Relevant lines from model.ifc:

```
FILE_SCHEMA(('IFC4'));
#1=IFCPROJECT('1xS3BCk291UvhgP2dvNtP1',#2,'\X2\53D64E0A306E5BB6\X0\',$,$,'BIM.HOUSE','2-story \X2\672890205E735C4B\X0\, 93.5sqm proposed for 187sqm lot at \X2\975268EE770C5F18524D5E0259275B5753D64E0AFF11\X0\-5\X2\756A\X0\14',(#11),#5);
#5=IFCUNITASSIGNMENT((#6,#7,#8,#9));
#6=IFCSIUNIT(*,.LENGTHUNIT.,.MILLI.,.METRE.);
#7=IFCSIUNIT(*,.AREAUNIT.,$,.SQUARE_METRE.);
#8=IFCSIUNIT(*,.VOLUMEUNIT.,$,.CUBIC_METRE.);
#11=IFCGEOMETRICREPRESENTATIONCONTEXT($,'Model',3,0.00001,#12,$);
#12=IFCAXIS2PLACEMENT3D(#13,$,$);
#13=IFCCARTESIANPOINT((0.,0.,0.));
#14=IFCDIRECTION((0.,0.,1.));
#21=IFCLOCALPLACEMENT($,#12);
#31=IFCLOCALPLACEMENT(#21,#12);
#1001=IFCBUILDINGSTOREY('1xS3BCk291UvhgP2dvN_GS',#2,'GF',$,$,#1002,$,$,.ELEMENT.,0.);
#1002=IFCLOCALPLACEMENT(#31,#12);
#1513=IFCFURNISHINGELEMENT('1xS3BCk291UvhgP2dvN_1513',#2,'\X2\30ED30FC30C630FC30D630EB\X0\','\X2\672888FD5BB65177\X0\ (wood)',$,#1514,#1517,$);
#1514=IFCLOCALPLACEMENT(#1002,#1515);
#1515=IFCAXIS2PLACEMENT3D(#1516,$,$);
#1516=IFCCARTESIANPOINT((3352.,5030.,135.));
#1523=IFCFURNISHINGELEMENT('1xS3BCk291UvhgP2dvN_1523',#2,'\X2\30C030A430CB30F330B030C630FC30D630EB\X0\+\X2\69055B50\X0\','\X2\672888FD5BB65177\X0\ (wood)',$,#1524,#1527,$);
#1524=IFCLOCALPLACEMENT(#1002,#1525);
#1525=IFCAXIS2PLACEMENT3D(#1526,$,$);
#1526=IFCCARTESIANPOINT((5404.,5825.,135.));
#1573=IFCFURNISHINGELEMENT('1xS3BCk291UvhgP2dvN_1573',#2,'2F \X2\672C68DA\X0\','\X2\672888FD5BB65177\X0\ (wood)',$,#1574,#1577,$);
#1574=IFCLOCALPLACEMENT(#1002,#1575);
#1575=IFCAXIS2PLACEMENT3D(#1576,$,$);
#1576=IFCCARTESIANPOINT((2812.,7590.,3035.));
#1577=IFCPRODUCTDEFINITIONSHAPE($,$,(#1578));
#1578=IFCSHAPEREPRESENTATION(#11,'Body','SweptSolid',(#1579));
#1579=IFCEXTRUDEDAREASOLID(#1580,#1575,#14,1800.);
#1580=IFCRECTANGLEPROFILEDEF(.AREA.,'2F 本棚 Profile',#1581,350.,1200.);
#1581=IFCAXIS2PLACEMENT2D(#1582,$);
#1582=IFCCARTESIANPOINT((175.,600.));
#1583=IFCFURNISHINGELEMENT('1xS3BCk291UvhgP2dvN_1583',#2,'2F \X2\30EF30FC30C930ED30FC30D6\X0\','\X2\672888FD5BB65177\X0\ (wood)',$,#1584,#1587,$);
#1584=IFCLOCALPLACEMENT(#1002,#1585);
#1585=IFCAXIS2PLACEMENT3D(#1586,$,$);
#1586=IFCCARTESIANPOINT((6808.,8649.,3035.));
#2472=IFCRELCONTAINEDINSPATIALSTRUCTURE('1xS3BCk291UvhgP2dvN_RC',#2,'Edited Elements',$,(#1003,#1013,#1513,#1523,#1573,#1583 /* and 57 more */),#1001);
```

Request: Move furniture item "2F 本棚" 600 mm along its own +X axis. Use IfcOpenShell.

```python
import ifcopenshell
import ifcopenshell.api.geometry
import ifcopenshell.util.placement
import ifcopenshell.util.unit

model = ifcopenshell.open("model.ifc")
unit_scale = ifcopenshell.util.unit.calculate_unit_scale(model)

item = model.by_guid("1xS3BCk291UvhgP2dvN_1573")
matrix = ifcopenshell.util.placement.get_local_placement(item.ObjectPlacement)
matrix[:3, 3] += matrix[:3, 0] * 0.6 / unit_scale
ifcopenshell.api.geometry.edit_object_placement(model, product=item, matrix=matrix, is_si=False)

print(ifcopenshell.util.placement.get_local_placement(item.ObjectPlacement).round(3) + 0.0)

model.write("model_v2.ifc")
```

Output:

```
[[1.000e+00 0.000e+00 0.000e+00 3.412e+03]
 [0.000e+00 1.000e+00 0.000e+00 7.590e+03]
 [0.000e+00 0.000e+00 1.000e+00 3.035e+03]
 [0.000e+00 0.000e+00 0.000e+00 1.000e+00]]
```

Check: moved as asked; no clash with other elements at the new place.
